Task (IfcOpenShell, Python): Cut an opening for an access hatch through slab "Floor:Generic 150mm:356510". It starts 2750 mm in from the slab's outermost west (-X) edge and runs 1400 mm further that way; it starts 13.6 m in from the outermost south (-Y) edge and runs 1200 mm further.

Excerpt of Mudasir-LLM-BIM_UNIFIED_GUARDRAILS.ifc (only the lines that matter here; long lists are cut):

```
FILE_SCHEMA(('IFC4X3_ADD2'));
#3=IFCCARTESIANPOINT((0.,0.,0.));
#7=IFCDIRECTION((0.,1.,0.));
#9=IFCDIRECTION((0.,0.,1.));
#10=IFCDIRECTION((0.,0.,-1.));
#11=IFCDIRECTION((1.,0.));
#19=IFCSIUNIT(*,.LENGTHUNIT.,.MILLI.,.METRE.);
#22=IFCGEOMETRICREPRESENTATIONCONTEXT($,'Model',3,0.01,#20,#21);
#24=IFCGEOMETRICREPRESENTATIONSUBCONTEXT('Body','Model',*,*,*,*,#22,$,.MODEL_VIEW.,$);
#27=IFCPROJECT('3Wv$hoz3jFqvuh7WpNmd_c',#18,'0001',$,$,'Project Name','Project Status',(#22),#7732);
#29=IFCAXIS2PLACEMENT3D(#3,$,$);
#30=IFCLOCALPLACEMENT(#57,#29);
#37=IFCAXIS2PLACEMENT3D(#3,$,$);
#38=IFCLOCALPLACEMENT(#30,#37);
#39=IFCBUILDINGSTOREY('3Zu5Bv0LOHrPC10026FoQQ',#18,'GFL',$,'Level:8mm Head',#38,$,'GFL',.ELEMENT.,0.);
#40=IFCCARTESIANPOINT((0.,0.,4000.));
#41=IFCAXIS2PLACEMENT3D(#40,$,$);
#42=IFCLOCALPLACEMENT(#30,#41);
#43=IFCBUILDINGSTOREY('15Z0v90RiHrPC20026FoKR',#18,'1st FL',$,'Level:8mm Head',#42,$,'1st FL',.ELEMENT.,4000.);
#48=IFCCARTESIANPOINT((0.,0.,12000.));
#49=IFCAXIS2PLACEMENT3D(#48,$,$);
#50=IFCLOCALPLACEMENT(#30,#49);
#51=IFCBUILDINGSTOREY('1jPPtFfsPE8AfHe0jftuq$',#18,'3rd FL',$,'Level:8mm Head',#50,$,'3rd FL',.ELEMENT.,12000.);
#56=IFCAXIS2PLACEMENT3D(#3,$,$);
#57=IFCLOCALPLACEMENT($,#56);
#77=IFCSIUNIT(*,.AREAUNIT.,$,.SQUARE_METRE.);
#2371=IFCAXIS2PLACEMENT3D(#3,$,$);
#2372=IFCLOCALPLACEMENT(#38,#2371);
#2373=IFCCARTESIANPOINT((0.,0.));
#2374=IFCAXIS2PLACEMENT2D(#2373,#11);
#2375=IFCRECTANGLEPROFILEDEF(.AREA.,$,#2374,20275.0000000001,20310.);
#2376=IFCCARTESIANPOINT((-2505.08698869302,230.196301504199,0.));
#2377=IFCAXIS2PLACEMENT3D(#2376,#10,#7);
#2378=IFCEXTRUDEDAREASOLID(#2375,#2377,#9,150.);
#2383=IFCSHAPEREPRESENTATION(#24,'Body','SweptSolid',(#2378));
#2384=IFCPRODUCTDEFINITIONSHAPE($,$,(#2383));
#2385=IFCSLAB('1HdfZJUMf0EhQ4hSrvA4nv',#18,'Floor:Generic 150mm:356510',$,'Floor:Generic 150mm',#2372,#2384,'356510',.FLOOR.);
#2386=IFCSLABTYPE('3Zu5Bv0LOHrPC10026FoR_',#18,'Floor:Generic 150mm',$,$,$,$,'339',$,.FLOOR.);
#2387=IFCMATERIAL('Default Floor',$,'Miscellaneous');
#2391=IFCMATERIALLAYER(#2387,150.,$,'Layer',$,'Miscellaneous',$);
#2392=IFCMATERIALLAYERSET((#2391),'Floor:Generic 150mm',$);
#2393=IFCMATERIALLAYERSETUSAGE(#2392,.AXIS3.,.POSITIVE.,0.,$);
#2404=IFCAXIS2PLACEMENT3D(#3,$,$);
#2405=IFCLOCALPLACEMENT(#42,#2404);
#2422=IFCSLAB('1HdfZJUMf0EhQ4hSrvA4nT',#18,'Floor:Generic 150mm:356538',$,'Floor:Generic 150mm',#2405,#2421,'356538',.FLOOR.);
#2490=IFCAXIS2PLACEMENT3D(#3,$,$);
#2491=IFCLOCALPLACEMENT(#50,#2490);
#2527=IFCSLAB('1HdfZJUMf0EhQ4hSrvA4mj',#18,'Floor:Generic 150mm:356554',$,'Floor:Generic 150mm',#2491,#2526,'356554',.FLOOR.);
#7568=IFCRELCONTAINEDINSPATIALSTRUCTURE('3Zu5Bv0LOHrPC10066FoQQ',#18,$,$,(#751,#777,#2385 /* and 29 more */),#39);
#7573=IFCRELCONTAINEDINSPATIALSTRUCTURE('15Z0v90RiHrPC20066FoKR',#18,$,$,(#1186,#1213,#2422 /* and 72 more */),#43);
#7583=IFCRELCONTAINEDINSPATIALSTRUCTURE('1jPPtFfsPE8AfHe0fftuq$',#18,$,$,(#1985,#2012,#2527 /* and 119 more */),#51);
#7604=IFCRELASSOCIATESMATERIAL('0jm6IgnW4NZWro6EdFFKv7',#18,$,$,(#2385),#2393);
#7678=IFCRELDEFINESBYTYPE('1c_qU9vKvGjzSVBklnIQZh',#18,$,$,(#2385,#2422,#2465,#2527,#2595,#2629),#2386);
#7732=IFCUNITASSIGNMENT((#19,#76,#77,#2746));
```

```python
import numpy as np
import ifcopenshell
import ifcopenshell.api.feature
import ifcopenshell.api.geometry
import ifcopenshell.api.root
import ifcopenshell.geom
import ifcopenshell.util.placement
import ifcopenshell.util.representation
import ifcopenshell.util.shape
import ifcopenshell.util.unit

model = ifcopenshell.open("Mudasir-LLM-BIM_UNIFIED_GUARDRAILS.ifc")
unit_scale = ifcopenshell.util.unit.calculate_unit_scale(model)
settings = ifcopenshell.geom.settings()


def volume(element):
    """Net volume in cubic metres, openings subtracted."""
    shape = ifcopenshell.geom.create_shape(settings, element)
    return ifcopenshell.util.shape.get_volume(shape.geometry)


slab = model.by_guid("1HdfZJUMf0EhQ4hSrvA4nv")
before = volume(slab)

# Extent in the slab's own axes, in metres. The edges named are its -X and -Y sides.
slab_shape = ifcopenshell.geom.create_shape(settings, slab)
vertices = ifcopenshell.util.shape.get_vertices(slab_shape.geometry)
x_min, y_min, bottom = vertices.min(axis=0)
top = vertices[:, 2].max()

opening = ifcopenshell.api.root.create_entity(model, ifc_class="IfcOpeningElement", name="Access hatch opening", predefined_type="OPENING")
context = ifcopenshell.util.representation.get_context(model, "Model", "Body", "MODEL_VIEW")
width, depth = 1.4, 1.2
outline = [(0.0, 0.0), (width, 0.0), (width, depth), (0.0, depth), (0.0, 0.0)]
# Overshoot both faces by 50 mm so the cut is clean.
shape = ifcopenshell.api.geometry.add_slab_representation(
    model, context=context, depth=top - bottom + 0.1, polyline=outline
)
ifcopenshell.api.geometry.assign_representation(model, product=opening, representation=shape)

matrix = ifcopenshell.util.placement.get_local_placement(slab.ObjectPlacement)
matrix[:, 3] = matrix @ np.append(np.array([x_min + 2.75, y_min + 13.6, bottom - 0.05]) / unit_scale, 1.0)
ifcopenshell.api.geometry.edit_object_placement(model, product=opening, matrix=matrix, is_si=False)
ifcopenshell.api.feature.add_feature(model, feature=opening, element=slab)

after = volume(slab)

print(f"slab volume {before:.3f} -> {after:.3f} m3")

model.write("Mudasir-LLM-BIM_UNIFIED_GUARDRAILS-out.ifc")
```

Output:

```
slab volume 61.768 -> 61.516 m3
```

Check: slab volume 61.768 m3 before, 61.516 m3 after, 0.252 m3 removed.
